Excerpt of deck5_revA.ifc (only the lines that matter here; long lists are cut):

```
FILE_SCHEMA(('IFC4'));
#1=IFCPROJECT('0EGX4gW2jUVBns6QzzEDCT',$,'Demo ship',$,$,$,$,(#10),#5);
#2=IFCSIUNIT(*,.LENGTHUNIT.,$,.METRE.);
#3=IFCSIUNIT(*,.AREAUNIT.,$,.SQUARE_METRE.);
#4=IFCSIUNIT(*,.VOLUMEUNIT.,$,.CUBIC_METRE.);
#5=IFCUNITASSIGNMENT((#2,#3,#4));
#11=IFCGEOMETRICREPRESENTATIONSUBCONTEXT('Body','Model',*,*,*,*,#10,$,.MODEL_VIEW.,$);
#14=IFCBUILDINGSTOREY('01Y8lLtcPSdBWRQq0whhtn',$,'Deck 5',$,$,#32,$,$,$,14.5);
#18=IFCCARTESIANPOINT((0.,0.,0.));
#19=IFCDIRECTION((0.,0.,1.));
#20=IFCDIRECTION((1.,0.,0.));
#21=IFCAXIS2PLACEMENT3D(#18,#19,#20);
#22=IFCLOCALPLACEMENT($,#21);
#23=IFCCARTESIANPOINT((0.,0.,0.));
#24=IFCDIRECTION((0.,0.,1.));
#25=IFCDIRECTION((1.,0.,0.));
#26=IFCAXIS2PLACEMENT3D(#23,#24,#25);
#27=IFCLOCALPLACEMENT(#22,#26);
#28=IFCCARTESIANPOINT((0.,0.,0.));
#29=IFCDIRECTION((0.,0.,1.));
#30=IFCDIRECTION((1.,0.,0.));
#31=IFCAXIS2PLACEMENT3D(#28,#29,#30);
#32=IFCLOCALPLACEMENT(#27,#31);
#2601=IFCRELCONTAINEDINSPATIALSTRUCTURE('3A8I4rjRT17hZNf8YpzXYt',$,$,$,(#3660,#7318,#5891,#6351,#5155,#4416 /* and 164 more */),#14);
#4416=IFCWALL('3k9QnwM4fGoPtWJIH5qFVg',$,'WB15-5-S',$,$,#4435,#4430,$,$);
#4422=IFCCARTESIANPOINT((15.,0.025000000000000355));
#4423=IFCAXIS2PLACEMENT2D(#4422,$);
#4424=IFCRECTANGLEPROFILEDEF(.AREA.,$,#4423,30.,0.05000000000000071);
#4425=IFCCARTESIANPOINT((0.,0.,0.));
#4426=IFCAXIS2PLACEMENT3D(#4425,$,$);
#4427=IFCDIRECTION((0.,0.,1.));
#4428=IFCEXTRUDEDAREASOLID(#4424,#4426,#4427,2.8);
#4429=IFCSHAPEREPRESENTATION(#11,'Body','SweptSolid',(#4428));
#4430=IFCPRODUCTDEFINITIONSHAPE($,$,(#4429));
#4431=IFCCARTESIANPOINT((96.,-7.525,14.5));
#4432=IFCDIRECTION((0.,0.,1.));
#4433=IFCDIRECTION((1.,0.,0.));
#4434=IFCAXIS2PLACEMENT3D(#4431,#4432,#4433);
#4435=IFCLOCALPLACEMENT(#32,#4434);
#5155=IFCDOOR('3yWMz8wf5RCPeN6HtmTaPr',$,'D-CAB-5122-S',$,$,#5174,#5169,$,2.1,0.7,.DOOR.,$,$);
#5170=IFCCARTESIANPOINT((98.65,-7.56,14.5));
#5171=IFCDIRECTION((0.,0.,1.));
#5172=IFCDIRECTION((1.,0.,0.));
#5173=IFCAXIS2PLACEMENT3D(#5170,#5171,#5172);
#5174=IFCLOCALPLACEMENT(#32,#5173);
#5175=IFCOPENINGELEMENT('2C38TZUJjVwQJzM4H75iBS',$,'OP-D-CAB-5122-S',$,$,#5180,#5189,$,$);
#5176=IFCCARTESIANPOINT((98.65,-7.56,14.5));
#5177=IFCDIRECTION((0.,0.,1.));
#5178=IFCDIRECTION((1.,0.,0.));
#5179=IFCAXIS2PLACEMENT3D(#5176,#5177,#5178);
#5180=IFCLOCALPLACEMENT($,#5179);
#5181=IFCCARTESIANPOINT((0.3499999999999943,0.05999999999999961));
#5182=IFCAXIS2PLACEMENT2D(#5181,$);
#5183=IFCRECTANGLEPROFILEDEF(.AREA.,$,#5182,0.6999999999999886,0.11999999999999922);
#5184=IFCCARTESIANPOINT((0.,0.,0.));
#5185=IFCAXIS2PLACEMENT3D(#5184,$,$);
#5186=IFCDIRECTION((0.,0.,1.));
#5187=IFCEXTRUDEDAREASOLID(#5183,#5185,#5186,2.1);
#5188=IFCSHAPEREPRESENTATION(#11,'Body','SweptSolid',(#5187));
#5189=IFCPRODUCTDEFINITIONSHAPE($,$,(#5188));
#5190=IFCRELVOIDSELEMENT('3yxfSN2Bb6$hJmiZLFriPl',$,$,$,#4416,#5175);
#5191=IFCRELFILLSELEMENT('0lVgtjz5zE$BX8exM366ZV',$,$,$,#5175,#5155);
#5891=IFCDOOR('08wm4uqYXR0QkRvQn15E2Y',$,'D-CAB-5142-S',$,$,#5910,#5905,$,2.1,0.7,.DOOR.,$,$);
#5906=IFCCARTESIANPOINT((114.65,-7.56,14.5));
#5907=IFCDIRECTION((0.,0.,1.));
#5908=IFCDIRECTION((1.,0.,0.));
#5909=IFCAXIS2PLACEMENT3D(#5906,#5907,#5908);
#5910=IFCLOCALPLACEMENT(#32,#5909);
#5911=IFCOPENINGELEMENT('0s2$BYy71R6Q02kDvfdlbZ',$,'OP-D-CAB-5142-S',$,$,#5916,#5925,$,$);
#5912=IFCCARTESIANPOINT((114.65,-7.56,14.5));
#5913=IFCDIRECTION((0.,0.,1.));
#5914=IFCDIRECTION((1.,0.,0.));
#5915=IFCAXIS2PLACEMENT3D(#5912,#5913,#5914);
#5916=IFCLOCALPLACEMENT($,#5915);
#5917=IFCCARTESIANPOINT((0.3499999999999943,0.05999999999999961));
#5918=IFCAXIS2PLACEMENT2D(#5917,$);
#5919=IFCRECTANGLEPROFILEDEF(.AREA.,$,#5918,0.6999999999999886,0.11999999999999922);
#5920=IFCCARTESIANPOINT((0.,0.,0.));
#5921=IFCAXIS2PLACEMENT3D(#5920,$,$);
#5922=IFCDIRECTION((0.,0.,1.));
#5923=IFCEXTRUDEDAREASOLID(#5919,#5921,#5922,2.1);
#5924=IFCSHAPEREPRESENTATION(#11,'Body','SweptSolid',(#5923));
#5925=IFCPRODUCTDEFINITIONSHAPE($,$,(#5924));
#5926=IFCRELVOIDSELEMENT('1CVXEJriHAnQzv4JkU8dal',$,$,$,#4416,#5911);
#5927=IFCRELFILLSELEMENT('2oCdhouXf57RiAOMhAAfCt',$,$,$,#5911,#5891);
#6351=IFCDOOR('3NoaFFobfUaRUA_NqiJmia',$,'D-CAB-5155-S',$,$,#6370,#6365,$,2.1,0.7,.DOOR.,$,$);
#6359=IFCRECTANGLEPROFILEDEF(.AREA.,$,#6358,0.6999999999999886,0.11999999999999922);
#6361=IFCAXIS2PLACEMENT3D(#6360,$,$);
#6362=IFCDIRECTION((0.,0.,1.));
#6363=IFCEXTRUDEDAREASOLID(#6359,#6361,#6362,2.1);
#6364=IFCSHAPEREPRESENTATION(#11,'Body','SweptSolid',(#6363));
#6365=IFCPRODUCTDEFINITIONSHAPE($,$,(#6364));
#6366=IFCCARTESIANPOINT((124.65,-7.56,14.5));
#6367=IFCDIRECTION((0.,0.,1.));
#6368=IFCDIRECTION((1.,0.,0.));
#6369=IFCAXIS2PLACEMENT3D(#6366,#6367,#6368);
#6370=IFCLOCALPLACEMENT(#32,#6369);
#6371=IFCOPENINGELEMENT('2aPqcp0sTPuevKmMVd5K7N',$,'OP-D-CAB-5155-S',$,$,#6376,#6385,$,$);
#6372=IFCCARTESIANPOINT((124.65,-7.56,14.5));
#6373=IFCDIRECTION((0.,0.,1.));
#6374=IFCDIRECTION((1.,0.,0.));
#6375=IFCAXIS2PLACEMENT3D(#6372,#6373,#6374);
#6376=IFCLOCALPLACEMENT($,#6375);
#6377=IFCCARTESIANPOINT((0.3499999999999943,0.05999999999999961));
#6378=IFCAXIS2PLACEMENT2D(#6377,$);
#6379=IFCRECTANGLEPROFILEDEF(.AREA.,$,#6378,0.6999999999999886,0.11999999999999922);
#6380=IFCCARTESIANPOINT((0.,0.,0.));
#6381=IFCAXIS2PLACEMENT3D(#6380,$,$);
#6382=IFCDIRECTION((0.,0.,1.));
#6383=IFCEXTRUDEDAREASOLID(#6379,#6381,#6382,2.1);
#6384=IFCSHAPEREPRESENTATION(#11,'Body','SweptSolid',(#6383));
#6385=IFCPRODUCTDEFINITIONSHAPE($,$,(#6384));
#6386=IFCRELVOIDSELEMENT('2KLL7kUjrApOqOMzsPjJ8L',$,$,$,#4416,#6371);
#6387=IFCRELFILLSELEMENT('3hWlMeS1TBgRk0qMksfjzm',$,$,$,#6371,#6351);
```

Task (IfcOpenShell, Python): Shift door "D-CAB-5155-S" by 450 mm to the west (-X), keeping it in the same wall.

```python
import ifcopenshell
import ifcopenshell.api.geometry
import ifcopenshell.util.placement
import ifcopenshell.util.unit

model = ifcopenshell.open("deck5_revA.ifc")
unit_scale = ifcopenshell.util.unit.calculate_unit_scale(model)

door = model.by_id(6351)
opening = door.FillsVoids[0].RelatingOpeningElement
wall = opening.VoidsElements[0].RelatingBuildingElement

wall_matrix = ifcopenshell.util.placement.get_local_placement(wall.ObjectPlacement)
shift = wall_matrix[:3, 0] * -0.45 / unit_scale
before = ifcopenshell.util.placement.get_local_placement(door.ObjectPlacement)[:3, 3].copy()

# The door is not placed relative to its opening, so move both.
for product in (opening, door):
    matrix = ifcopenshell.util.placement.get_local_placement(product.ObjectPlacement)
    matrix[:3, 3] += shift
    ifcopenshell.api.geometry.edit_object_placement(model, product=product, matrix=matrix, is_si=False)

after = ifcopenshell.util.placement.get_local_placement(door.ObjectPlacement)[:3, 3]
print("door moved by", (after - before).round(3) + 0.0)

model.write("deck5_revA_edited.ifc")
```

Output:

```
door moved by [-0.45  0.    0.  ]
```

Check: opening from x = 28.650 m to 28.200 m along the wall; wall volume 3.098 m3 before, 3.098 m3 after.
